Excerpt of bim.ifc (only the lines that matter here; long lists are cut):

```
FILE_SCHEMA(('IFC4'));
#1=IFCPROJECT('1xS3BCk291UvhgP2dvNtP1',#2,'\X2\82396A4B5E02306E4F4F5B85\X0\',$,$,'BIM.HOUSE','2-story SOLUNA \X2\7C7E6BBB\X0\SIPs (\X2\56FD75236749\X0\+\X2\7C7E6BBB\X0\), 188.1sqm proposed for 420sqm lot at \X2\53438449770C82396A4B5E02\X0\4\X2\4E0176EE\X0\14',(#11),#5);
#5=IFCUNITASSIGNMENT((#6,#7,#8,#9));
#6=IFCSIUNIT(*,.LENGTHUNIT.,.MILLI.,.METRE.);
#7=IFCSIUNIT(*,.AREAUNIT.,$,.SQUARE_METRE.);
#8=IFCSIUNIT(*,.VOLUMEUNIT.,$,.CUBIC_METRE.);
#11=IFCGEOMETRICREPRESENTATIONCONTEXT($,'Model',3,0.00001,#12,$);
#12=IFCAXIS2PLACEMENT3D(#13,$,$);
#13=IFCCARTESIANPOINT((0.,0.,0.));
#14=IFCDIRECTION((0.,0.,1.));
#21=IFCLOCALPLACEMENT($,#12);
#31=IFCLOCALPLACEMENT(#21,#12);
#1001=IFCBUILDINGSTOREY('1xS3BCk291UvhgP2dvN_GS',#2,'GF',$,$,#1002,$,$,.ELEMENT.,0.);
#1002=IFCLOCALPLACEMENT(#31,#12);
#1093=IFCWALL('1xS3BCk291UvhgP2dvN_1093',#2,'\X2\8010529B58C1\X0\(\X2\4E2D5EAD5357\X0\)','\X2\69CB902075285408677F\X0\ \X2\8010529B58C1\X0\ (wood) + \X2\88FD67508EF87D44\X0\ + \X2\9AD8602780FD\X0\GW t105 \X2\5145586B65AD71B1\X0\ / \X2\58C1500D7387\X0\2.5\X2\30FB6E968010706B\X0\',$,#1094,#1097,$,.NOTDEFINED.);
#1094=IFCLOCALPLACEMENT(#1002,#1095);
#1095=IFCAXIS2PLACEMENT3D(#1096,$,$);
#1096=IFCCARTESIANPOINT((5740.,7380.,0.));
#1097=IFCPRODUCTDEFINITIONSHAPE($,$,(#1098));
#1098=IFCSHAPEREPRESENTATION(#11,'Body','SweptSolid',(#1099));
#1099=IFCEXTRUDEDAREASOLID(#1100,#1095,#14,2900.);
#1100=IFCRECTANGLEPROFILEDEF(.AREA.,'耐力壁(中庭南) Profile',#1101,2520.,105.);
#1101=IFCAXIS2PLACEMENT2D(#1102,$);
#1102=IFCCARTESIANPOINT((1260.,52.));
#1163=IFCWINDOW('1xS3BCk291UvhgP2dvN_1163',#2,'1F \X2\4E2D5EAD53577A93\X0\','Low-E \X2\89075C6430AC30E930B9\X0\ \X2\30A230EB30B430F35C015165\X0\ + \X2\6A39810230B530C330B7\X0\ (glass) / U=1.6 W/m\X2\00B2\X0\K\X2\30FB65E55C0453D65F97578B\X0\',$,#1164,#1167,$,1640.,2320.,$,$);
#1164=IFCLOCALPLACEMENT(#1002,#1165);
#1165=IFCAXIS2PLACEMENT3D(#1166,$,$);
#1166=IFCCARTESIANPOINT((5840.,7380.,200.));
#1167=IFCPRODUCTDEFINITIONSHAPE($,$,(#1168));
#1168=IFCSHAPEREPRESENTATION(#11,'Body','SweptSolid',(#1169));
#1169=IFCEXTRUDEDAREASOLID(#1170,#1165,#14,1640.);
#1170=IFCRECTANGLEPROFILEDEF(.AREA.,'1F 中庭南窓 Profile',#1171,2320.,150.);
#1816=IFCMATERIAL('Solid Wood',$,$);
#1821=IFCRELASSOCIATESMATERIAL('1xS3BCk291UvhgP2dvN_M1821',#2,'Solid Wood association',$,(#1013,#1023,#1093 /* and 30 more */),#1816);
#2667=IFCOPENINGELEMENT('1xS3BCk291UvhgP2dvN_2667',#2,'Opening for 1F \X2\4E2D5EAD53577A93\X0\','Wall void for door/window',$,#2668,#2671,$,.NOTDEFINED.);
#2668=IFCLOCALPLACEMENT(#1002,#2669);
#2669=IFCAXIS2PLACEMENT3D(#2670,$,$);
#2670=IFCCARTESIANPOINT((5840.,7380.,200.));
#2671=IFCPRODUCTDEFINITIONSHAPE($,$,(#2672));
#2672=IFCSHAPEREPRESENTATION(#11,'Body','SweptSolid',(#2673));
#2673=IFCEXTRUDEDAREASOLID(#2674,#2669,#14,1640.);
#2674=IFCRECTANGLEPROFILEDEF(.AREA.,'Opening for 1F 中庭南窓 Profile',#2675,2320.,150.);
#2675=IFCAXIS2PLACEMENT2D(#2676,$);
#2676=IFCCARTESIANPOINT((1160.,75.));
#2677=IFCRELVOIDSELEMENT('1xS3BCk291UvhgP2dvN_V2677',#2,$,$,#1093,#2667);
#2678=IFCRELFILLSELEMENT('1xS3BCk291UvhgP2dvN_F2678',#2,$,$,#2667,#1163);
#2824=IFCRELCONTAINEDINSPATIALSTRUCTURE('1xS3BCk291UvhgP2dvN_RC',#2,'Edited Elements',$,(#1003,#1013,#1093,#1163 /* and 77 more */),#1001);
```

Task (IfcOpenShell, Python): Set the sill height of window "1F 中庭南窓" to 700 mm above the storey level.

```python
import numpy as np
import ifcopenshell
import ifcopenshell.api.geometry
import ifcopenshell.geom
import ifcopenshell.util.element
import ifcopenshell.util.placement
import ifcopenshell.util.shape
import ifcopenshell.util.unit

model = ifcopenshell.open("bim.ifc")
unit_scale = ifcopenshell.util.unit.calculate_unit_scale(model)

window = model.by_id(1163)
opening = window.FillsVoids[0].RelatingOpeningElement
storey = ifcopenshell.util.element.get_container(window, ifc_class="IfcBuildingStorey")
level = ifcopenshell.util.placement.get_local_placement(storey.ObjectPlacement)[2, 3]

# The opening's origin need not be at the sill, so measure its lowest point.
shape = ifcopenshell.geom.create_shape(ifcopenshell.geom.settings(), opening)
bottom = ifcopenshell.util.shape.get_shape_bottom_elevation(shape, shape.geometry) / unit_scale
dz = level + 0.7 / unit_scale - bottom

shift = np.array([0.0, 0.0, dz])
# The window is not placed relative to its opening, so move both.
for product in (opening, window):
    matrix = ifcopenshell.util.placement.get_local_placement(product.ObjectPlacement)
    matrix[:3, 3] += shift
    ifcopenshell.api.geometry.edit_object_placement(model, product=product, matrix=matrix, is_si=False)

print(f"moved by {dz * unit_scale:+.3f} m")

model.write("bim_updated.ifc")
```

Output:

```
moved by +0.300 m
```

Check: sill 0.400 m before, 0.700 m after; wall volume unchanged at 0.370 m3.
